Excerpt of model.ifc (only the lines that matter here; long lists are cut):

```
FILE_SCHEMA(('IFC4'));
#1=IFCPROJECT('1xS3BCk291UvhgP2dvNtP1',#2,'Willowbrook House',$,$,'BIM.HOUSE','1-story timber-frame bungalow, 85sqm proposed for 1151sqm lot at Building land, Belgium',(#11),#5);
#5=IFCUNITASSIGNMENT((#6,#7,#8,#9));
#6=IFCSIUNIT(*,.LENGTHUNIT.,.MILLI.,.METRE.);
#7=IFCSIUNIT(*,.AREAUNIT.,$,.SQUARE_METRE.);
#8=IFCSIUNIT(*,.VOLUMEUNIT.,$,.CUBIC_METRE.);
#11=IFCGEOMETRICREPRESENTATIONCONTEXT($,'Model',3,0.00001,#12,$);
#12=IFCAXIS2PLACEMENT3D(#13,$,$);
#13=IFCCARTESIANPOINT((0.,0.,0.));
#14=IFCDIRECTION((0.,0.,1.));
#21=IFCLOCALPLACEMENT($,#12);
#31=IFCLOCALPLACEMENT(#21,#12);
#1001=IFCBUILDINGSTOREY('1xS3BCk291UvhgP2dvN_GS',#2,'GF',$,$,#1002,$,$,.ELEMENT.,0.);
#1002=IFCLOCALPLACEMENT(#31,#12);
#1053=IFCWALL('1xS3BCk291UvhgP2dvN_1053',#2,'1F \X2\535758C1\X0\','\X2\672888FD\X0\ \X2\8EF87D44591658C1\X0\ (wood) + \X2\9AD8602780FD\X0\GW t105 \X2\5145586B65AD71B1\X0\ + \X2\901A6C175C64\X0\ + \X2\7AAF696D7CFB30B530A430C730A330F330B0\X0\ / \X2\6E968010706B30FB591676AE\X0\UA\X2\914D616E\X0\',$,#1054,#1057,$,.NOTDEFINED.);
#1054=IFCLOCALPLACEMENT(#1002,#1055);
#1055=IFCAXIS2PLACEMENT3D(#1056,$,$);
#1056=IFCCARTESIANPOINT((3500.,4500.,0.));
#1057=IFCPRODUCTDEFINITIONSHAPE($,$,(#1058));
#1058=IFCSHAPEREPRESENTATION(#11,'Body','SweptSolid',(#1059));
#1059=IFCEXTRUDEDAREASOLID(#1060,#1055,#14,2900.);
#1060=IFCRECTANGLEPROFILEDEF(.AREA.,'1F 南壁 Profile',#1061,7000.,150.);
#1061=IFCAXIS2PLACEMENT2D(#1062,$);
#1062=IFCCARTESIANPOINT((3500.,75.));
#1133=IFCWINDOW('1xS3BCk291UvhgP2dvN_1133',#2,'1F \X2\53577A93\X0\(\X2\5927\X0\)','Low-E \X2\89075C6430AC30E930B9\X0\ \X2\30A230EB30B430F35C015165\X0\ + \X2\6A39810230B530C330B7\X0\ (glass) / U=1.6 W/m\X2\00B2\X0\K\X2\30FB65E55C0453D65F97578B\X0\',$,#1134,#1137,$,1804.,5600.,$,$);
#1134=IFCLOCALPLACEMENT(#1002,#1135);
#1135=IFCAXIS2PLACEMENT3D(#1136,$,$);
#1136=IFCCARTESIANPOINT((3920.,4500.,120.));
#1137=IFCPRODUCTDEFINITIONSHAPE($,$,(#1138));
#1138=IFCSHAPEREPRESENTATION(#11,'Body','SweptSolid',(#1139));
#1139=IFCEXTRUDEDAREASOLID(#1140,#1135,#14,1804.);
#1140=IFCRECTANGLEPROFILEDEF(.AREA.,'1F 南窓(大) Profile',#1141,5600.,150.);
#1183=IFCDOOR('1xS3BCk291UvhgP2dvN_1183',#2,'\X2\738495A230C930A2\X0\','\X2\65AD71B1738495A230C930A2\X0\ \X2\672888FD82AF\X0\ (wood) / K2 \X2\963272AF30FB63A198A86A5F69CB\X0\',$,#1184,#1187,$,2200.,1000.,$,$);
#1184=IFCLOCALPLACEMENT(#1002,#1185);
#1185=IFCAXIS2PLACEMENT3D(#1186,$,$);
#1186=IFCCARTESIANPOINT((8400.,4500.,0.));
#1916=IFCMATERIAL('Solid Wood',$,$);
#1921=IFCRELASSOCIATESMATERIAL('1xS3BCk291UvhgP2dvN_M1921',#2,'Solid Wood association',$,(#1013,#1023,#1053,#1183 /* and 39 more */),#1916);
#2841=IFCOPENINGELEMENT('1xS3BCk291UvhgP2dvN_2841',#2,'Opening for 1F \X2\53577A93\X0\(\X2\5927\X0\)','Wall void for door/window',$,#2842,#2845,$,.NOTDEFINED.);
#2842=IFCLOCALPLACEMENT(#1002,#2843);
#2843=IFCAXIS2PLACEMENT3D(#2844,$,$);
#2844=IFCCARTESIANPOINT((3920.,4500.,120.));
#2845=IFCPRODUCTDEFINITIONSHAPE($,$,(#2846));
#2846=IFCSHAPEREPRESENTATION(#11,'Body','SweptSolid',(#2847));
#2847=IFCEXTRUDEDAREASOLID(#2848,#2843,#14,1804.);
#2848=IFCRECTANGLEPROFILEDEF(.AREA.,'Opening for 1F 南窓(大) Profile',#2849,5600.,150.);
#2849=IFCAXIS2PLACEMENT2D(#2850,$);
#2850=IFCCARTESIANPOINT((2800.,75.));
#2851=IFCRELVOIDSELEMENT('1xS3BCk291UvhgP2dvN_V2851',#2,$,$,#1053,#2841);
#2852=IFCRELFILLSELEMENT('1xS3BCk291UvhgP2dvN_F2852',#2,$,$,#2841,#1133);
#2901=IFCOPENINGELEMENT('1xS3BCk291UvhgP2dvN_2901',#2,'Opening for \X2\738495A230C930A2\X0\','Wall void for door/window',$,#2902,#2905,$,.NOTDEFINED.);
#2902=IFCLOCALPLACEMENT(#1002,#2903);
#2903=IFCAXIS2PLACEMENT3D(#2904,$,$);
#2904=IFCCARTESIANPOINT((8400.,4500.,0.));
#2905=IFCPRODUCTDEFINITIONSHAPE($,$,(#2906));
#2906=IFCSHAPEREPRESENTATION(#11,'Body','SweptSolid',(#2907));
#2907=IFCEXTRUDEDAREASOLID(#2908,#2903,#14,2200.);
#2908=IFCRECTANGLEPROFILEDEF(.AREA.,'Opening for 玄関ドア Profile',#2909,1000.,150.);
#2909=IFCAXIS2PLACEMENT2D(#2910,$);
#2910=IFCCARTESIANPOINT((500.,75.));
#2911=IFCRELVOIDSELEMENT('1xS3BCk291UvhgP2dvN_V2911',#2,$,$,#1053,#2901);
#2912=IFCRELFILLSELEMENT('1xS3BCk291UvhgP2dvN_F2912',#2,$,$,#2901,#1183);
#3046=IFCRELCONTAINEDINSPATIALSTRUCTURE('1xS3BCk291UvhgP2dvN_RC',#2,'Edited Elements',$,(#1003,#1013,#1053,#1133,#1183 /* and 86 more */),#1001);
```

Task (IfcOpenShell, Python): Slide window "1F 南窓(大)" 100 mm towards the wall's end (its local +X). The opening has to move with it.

```python
import ifcopenshell
import ifcopenshell.api.geometry
import ifcopenshell.util.placement

model = ifcopenshell.open("model.ifc")

window = model.by_guid("1xS3BCk291UvhgP2dvN_1133")
opening = window.FillsVoids[0].RelatingOpeningElement
wall = opening.VoidsElements[0].RelatingBuildingElement

wall_matrix = ifcopenshell.util.placement.get_local_placement(wall.ObjectPlacement)
shift = wall_matrix[:3, 0] * 100.0
before = ifcopenshell.util.placement.get_local_placement(window.ObjectPlacement)[:3, 3].copy()

# The window is not placed relative to its opening, so move both.
for product in (opening, window):
    matrix = ifcopenshell.util.placement.get_local_placement(product.ObjectPlacement)
    matrix[:3, 3] += shift
    ifcopenshell.api.geometry.edit_object_placement(model, product=product, matrix=matrix, is_si=False)

after = ifcopenshell.util.placement.get_local_placement(window.ObjectPlacement)[:3, 3]
print("window moved by", (after - before).round(3) + 0.0)

model.write("model-out.ifc")
```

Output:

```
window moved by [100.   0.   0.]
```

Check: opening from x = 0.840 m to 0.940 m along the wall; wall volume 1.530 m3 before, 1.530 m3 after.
